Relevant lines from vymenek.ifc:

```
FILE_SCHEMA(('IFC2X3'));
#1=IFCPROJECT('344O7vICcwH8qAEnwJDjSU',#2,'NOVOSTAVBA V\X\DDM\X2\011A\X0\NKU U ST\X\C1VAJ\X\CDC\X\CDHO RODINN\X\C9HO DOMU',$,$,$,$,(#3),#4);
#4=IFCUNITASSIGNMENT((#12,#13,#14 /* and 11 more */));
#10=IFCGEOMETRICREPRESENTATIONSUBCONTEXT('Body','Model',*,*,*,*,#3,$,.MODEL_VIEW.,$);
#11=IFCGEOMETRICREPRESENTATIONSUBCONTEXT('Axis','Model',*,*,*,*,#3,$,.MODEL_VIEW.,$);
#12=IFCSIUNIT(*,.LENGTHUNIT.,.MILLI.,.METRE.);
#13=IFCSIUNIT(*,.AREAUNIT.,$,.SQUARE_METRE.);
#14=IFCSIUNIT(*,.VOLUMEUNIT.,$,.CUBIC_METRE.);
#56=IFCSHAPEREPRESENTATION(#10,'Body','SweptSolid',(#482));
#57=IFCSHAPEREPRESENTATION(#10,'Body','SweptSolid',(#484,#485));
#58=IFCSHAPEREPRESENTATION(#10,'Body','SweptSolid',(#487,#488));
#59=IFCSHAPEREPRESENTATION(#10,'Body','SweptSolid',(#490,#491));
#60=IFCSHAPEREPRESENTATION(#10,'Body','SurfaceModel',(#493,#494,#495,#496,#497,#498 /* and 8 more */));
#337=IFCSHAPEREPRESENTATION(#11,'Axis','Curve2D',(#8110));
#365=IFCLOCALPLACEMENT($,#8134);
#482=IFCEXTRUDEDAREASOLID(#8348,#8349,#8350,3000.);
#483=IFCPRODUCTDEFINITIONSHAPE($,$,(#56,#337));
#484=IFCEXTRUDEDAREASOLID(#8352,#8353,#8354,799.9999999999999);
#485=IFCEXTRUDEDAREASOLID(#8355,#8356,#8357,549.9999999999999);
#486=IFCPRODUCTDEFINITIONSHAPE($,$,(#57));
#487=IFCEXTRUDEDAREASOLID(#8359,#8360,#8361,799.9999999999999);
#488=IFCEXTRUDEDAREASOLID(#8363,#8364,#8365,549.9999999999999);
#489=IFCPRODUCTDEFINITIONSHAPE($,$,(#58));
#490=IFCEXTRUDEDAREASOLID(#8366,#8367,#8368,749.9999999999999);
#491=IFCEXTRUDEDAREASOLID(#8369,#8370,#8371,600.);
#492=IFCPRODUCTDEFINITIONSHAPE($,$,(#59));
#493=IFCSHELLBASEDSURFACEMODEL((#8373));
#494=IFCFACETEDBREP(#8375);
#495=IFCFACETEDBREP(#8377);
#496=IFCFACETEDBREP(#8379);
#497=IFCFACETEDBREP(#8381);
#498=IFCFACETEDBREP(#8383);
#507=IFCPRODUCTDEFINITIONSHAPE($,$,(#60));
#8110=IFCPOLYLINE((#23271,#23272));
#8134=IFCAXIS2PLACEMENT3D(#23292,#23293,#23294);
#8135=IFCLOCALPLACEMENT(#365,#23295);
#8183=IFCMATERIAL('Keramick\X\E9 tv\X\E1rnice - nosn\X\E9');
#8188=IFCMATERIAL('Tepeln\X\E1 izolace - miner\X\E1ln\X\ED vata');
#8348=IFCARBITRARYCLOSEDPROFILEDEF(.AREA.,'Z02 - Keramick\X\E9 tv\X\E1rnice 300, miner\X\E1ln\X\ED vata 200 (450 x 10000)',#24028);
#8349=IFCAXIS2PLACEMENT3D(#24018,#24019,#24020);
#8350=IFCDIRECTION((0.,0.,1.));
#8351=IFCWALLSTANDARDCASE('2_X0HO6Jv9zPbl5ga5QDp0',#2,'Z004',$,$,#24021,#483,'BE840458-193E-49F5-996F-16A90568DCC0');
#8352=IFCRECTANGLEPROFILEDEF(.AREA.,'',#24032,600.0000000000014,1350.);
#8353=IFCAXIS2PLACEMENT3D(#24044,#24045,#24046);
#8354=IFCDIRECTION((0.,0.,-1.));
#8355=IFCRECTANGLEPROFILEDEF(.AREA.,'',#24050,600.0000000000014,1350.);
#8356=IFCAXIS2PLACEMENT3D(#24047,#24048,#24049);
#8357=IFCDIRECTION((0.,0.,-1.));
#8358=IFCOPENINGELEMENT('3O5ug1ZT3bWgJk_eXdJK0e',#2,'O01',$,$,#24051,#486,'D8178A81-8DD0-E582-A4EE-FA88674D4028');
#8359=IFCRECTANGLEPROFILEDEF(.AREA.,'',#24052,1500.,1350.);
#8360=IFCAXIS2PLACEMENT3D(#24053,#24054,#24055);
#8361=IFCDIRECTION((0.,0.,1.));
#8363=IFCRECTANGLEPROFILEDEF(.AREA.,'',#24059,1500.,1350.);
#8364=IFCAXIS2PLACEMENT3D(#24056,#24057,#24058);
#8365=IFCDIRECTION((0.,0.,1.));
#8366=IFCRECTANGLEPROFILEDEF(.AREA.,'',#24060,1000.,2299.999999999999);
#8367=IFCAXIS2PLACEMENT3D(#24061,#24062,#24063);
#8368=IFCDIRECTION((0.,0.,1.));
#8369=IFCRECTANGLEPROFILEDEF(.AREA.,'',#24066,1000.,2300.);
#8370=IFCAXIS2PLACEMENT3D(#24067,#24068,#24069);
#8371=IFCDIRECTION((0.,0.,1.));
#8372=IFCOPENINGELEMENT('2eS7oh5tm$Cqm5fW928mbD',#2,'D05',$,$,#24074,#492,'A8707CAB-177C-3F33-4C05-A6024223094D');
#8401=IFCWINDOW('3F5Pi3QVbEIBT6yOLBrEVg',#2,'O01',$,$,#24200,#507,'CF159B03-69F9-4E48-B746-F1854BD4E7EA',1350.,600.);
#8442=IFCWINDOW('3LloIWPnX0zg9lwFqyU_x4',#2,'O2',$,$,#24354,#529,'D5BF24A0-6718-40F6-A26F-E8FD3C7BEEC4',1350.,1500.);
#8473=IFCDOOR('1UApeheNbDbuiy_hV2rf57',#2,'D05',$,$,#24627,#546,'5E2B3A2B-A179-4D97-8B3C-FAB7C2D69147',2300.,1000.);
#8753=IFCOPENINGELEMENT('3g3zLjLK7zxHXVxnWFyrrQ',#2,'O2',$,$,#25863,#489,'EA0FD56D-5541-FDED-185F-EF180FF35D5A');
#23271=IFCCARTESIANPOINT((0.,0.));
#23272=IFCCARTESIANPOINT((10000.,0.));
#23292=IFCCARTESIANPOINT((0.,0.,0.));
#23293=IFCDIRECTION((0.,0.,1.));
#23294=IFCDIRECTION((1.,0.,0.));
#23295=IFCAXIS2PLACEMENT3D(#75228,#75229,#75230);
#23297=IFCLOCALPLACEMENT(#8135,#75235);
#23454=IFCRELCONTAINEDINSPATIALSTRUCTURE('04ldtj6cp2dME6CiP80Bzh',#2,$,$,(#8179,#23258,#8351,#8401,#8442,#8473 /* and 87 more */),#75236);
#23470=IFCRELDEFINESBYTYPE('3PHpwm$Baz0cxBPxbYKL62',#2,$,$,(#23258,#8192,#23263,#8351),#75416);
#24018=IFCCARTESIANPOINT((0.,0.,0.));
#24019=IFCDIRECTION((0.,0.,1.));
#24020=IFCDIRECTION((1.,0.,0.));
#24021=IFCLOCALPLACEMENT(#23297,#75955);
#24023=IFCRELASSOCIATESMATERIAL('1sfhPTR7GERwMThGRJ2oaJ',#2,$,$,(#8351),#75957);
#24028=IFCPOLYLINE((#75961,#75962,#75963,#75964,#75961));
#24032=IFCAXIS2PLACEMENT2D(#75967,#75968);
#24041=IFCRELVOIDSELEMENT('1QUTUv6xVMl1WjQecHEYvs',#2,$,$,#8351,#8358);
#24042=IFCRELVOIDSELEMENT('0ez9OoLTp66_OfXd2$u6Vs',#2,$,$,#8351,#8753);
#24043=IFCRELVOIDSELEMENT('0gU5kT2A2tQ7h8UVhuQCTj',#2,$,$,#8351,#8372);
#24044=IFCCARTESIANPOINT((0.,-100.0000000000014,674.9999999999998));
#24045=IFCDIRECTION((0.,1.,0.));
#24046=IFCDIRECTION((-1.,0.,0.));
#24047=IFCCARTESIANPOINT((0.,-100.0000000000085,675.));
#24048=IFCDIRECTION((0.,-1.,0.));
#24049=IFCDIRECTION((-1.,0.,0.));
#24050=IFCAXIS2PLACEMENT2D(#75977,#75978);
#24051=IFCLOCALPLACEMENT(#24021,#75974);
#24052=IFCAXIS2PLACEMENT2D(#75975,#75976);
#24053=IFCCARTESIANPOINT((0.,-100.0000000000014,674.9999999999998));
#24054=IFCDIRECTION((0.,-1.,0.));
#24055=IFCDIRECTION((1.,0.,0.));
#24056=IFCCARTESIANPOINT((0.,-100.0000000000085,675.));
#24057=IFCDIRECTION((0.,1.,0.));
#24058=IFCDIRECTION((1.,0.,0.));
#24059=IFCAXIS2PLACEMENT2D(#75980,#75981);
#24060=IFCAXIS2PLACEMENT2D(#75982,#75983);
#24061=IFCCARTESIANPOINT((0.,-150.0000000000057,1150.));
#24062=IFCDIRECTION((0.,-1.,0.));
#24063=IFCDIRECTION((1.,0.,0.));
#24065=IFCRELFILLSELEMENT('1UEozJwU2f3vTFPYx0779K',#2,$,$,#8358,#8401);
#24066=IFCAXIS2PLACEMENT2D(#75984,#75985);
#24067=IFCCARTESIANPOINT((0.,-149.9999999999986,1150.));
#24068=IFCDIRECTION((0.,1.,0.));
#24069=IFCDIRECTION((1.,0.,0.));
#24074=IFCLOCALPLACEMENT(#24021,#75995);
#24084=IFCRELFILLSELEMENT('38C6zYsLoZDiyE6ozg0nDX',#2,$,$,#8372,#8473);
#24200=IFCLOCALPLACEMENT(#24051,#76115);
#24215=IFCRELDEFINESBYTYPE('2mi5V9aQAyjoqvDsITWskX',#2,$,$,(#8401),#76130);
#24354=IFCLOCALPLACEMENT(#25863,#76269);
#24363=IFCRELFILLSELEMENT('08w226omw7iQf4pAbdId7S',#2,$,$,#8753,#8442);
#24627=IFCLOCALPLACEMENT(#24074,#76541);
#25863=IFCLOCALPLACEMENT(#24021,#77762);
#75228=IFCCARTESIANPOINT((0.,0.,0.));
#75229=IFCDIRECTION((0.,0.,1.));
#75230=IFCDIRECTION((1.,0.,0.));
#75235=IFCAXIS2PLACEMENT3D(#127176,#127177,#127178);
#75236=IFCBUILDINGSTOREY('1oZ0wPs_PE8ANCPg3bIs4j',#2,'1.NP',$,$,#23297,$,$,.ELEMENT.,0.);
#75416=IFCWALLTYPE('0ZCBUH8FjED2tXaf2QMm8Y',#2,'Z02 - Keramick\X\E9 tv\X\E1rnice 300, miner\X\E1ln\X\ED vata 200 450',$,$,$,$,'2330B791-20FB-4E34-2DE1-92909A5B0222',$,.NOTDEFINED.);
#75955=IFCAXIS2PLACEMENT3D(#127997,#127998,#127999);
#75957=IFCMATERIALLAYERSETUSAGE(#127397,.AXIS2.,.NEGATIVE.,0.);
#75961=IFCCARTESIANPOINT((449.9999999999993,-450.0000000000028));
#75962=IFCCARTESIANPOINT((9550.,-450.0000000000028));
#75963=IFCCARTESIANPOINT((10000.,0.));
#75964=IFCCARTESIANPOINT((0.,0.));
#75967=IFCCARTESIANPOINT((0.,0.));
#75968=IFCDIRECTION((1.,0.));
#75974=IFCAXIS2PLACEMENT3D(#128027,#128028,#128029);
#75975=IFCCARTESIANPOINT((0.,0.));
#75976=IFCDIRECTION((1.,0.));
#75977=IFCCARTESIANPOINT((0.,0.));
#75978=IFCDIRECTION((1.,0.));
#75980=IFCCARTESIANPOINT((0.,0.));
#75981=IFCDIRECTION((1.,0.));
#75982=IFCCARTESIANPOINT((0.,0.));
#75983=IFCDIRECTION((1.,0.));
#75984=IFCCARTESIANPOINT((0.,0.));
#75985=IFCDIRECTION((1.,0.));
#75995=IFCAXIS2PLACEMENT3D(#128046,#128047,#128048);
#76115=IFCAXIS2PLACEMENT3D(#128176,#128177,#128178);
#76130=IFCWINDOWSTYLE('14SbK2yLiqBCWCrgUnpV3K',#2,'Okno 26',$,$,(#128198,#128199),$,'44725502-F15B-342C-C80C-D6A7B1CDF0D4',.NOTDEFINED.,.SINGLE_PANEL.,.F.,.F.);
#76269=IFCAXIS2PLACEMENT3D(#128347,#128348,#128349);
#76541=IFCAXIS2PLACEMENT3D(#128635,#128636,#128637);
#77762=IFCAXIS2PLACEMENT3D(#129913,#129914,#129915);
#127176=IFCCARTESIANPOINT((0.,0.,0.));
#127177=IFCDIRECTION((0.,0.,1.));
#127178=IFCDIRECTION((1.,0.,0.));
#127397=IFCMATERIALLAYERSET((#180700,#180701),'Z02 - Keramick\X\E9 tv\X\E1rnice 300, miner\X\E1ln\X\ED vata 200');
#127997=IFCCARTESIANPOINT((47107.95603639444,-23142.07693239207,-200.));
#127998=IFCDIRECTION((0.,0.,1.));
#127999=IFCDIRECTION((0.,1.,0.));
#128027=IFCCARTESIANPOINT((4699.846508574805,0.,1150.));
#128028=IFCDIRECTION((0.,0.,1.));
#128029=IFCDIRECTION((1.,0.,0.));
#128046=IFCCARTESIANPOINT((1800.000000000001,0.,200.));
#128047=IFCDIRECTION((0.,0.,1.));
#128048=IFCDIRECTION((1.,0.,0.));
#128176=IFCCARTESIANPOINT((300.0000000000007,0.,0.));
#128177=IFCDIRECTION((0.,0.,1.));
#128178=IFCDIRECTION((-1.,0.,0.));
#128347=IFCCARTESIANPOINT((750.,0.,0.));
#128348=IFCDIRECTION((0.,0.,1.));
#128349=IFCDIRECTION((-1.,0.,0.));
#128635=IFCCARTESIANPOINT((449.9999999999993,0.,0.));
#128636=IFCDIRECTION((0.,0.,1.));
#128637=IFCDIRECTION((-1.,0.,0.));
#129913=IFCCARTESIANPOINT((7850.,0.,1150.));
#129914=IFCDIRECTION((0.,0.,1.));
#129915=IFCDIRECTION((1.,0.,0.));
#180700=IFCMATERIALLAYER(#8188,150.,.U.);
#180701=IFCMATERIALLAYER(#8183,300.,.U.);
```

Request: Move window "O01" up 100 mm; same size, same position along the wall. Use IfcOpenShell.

```python
import numpy as np
import ifcopenshell
import ifcopenshell.api.geometry
import ifcopenshell.util.placement
import ifcopenshell.util.unit

model = ifcopenshell.open("vymenek.ifc")
unit_scale = ifcopenshell.util.unit.calculate_unit_scale(model)

window = model.by_guid("3F5Pi3QVbEIBT6yOLBrEVg")
opening = window.FillsVoids[0].RelatingOpeningElement
dz = 100.0

shift = np.array([0.0, 0.0, dz])
# The window is placed relative to its opening, so it follows when the opening moves.
matrix = ifcopenshell.util.placement.get_local_placement(opening.ObjectPlacement)
matrix[:3, 3] += shift
ifcopenshell.api.geometry.edit_object_placement(
    model, product=opening, matrix=matrix, is_si=False, should_transform_children=True
)

print(f"moved by {dz * unit_scale:+.3f} m")

model.write("vymenek_updated.ifc")
```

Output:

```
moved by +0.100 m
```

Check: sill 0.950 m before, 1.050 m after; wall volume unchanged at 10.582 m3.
